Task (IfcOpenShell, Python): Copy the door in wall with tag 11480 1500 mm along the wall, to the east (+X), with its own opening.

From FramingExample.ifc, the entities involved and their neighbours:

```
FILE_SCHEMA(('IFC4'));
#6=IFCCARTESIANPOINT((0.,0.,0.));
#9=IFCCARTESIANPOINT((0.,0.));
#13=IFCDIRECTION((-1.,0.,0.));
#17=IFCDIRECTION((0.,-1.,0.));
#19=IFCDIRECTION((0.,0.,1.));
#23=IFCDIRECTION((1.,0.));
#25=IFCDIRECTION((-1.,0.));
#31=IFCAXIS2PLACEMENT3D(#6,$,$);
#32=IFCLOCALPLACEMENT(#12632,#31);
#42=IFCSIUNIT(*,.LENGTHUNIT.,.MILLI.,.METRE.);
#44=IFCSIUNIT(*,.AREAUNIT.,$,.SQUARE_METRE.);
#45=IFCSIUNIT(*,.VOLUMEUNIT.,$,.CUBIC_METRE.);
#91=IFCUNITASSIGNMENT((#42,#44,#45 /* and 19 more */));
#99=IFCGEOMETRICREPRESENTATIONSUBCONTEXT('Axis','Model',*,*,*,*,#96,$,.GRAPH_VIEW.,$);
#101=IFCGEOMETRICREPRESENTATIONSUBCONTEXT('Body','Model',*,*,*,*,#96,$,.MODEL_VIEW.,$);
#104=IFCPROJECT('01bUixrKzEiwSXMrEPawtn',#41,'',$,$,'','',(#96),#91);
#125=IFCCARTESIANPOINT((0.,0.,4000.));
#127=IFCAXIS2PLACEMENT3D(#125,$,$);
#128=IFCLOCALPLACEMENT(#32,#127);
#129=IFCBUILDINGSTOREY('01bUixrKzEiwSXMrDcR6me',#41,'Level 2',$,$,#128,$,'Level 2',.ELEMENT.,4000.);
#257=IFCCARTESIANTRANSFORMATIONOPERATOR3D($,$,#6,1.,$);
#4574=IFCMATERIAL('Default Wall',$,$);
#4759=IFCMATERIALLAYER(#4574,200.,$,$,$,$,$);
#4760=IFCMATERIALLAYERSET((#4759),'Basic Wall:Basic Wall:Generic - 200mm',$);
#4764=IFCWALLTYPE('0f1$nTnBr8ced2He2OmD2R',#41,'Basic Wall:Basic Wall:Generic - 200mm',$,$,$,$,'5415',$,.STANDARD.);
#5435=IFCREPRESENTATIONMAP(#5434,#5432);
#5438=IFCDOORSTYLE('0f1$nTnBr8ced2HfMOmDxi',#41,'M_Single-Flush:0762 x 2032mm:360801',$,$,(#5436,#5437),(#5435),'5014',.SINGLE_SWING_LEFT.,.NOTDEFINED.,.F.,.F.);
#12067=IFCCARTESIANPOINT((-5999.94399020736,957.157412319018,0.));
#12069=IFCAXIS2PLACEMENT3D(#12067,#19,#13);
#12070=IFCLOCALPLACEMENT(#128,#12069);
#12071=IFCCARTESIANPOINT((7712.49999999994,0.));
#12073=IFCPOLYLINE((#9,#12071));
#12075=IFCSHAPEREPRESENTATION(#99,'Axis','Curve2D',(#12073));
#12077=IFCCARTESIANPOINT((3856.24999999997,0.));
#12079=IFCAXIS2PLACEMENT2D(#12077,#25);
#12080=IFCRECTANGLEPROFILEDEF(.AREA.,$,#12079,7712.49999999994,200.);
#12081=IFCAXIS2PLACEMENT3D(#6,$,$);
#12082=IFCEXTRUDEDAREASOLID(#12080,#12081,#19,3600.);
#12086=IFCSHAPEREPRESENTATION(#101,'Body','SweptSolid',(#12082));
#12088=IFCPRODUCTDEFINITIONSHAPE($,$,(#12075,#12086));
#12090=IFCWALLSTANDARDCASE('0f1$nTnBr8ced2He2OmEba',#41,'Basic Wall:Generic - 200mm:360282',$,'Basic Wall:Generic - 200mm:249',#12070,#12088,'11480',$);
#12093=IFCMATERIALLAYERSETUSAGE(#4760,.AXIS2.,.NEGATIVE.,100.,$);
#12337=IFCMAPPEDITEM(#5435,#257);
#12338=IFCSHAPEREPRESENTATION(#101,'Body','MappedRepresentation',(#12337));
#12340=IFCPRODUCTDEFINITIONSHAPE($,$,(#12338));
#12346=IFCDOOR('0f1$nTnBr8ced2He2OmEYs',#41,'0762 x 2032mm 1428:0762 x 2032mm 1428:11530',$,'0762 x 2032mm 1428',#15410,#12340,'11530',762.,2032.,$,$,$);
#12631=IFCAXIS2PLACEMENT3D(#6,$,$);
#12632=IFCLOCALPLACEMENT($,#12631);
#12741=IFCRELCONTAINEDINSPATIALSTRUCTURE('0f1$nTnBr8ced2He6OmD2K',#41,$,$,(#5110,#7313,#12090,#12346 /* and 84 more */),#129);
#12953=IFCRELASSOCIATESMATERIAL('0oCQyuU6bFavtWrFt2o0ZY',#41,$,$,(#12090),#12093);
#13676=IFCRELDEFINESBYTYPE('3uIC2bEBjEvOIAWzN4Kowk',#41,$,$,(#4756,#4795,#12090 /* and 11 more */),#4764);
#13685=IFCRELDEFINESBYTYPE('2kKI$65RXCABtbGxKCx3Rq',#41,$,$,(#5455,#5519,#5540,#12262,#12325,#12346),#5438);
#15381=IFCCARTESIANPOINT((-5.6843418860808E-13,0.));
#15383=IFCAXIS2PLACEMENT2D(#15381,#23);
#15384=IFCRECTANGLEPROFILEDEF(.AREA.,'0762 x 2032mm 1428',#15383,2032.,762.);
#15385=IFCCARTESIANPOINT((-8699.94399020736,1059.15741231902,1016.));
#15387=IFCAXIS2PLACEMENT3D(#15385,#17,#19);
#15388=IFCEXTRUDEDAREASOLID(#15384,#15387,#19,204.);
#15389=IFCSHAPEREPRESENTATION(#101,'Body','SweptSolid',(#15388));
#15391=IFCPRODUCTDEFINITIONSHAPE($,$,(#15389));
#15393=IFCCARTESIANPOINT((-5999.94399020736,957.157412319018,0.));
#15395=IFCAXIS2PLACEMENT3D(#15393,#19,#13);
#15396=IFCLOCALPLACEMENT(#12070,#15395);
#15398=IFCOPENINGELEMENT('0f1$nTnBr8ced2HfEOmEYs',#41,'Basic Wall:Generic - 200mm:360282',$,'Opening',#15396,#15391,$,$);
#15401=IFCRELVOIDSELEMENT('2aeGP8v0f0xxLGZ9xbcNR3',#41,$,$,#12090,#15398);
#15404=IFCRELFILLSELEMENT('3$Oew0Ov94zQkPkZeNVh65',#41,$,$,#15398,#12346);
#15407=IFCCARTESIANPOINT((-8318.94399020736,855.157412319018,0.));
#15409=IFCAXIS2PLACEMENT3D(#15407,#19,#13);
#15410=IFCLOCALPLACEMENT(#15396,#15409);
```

```python
import ifcopenshell
import ifcopenshell.api.feature
import ifcopenshell.api.geometry
import ifcopenshell.api.root
import ifcopenshell.geom
import ifcopenshell.util.element
import ifcopenshell.util.placement
import ifcopenshell.util.shape
import ifcopenshell.util.unit

model = ifcopenshell.open("FramingExample.ifc")
unit_scale = ifcopenshell.util.unit.calculate_unit_scale(model)
settings = ifcopenshell.geom.settings()


def volume(element):
    """Net volume in cubic metres, openings subtracted."""
    shape = ifcopenshell.geom.create_shape(settings, element)
    return ifcopenshell.util.shape.get_volume(shape.geometry)


def reuse_history(source, copy):
    """copy_class also copies each property set's owner history, people and application; keep the originals."""
    for rel in copy.IsDefinedBy:
        if rel.is_a("IfcRelDefinesByProperties") and (history := rel.RelatingPropertyDefinition.OwnerHistory):
            rel.RelatingPropertyDefinition.OwnerHistory = source.OwnerHistory
            ifcopenshell.util.element.remove_deep2(model, history)


door = model.by_guid("0f1$nTnBr8ced2He2OmEYs")
opening = door.FillsVoids[0].RelatingOpeningElement
wall = opening.VoidsElements[0].RelatingBuildingElement
before = volume(wall)
shift = ifcopenshell.util.placement.get_local_placement(wall.ObjectPlacement)[:3, 0] * -1.5 / unit_scale

# copy_class copies the void relationship, type, container and properties, but no geometry.
new_opening = ifcopenshell.api.root.copy_class(model, product=opening)
new_opening.Representation = ifcopenshell.util.element.copy_deep(
    model, opening.Representation, exclude=["IfcGeometricRepresentationContext", "IfcRepresentationMap"]
)
new_opening.Name = "Basic Wall:Generic - 200mm"
new_door = ifcopenshell.api.root.copy_class(model, product=door)
new_door.Representation = ifcopenshell.util.element.copy_deep(
    model, door.Representation, exclude=["IfcGeometricRepresentationContext", "IfcRepresentationMap"]
)
new_door.Name = "0762 x 2032mm 1428:0762 x 2032mm 1428"
new_door.Tag = None
reuse_history(door, new_door)
ifcopenshell.api.feature.add_filling(model, opening=new_opening, element=new_door)

for old, new in ((opening, new_opening), (door, new_door)):
    matrix = ifcopenshell.util.placement.get_local_placement(old.ObjectPlacement)
    matrix[:3, 3] += shift
    ifcopenshell.api.geometry.edit_object_placement(model, product=new, matrix=matrix, is_si=False)

after = volume(wall)

print(f"wall volume {before:.3f} -> {after:.3f} m3")

model.write("FramingExample_edited.ifc")
```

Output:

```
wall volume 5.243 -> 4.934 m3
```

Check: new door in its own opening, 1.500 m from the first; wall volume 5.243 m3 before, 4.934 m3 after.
